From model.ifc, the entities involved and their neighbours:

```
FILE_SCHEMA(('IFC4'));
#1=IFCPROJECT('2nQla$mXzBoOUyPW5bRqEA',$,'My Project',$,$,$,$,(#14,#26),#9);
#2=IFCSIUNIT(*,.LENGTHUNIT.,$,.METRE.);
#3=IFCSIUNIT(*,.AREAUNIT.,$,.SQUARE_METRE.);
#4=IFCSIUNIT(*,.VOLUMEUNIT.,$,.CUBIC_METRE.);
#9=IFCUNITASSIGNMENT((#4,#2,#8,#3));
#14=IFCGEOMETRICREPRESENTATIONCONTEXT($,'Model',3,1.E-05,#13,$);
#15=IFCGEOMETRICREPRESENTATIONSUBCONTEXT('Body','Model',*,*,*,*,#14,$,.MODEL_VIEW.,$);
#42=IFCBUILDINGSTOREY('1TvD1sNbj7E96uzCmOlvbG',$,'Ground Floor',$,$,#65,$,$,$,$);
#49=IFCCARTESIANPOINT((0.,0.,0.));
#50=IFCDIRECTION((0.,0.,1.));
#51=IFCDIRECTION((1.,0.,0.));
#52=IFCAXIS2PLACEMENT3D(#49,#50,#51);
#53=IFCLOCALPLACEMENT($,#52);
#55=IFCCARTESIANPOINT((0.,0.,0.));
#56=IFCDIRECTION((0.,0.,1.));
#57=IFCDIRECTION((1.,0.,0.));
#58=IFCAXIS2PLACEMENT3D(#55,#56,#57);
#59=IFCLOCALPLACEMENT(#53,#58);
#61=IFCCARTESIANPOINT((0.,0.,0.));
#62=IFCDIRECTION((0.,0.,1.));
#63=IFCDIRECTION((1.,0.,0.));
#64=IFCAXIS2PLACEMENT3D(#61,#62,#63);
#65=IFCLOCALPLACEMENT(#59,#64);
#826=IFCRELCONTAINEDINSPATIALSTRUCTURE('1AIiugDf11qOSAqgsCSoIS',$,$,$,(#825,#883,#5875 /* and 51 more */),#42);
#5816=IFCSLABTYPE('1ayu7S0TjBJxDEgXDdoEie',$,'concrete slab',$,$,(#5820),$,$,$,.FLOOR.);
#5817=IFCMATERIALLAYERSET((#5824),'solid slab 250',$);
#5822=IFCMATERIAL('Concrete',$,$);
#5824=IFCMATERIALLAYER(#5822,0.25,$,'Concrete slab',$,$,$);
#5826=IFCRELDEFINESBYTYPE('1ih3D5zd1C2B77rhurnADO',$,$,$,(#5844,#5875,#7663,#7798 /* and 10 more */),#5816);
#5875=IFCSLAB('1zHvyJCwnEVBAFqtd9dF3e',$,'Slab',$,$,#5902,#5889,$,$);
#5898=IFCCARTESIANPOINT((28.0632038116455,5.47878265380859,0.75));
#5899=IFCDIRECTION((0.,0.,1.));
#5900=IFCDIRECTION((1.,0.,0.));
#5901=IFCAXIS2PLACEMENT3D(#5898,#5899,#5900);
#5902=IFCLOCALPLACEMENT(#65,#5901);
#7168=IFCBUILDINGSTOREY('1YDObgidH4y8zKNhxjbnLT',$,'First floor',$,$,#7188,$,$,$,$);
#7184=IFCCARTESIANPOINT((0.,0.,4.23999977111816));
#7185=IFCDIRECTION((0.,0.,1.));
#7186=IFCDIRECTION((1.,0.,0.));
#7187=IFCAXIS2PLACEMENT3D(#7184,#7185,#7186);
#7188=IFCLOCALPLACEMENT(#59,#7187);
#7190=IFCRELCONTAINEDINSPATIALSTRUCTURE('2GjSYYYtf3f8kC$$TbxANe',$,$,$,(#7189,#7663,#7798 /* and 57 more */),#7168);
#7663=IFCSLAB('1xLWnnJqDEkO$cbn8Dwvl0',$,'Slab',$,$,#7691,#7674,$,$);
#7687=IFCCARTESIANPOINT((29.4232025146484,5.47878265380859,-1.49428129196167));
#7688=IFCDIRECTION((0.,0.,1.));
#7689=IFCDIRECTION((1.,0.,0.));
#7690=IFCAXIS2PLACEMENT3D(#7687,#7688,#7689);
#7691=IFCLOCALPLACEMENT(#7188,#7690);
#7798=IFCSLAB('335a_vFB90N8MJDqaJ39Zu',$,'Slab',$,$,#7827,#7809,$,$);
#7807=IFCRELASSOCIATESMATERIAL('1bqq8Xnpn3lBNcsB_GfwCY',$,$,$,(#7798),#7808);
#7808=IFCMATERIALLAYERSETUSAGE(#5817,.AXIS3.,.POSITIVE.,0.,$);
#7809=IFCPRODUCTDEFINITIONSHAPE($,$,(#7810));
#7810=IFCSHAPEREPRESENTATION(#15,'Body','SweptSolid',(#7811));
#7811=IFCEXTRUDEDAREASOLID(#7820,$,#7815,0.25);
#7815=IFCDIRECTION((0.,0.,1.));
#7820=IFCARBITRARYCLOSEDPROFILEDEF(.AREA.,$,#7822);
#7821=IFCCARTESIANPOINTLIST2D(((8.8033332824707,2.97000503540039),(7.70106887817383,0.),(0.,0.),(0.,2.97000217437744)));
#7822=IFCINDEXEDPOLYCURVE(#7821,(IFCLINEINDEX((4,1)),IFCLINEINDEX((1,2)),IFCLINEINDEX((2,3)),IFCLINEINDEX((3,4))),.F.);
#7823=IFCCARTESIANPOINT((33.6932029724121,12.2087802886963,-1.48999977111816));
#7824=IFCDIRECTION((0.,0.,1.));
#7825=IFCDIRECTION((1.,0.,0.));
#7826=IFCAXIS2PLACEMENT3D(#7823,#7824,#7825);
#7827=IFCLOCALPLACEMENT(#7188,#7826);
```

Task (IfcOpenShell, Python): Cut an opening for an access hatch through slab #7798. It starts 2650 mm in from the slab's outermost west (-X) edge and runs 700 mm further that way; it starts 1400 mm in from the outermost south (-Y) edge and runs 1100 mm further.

```python
import numpy as np
import ifcopenshell
import ifcopenshell.api.feature
import ifcopenshell.api.geometry
import ifcopenshell.api.root
import ifcopenshell.geom
import ifcopenshell.util.placement
import ifcopenshell.util.representation
import ifcopenshell.util.shape
import ifcopenshell.util.unit

model = ifcopenshell.open("model.ifc")
unit_scale = ifcopenshell.util.unit.calculate_unit_scale(model)
settings = ifcopenshell.geom.settings()


def volume(element):
    """Net volume in cubic metres, openings subtracted."""
    shape = ifcopenshell.geom.create_shape(settings, element)
    return ifcopenshell.util.shape.get_volume(shape.geometry)


slab = model.by_guid("335a_vFB90N8MJDqaJ39Zu")
before = volume(slab)

# Extent in the slab's own axes, in metres. The edges named are its -X and -Y sides.
slab_shape = ifcopenshell.geom.create_shape(settings, slab)
vertices = ifcopenshell.util.shape.get_vertices(slab_shape.geometry)
x_min, y_min, bottom = vertices.min(axis=0)
top = vertices[:, 2].max()

opening = ifcopenshell.api.root.create_entity(model, ifc_class="IfcOpeningElement", name="Access hatch opening", predefined_type="OPENING")
context = ifcopenshell.util.representation.get_context(model, "Model", "Body", "MODEL_VIEW")
width, depth = 0.7, 1.1
outline = [(0.0, 0.0), (width, 0.0), (width, depth), (0.0, depth), (0.0, 0.0)]
# Overshoot both faces by 50 mm so the cut is clean.
shape = ifcopenshell.api.geometry.add_slab_representation(
    model, context=context, depth=top - bottom + 0.1, polyline=outline
)
ifcopenshell.api.geometry.assign_representation(model, product=opening, representation=shape)

matrix = ifcopenshell.util.placement.get_local_placement(slab.ObjectPlacement)
matrix[:, 3] = matrix @ np.append(np.array([x_min + 2.65, y_min + 1.4, bottom - 0.05]) / unit_scale, 1.0)
ifcopenshell.api.geometry.edit_object_placement(model, product=opening, matrix=matrix, is_si=False)
ifcopenshell.api.feature.add_feature(model, feature=opening, element=slab)

after = volume(slab)

print(f"slab volume {before:.3f} -> {after:.3f} m3")

model.write("model_v2.ifc")
```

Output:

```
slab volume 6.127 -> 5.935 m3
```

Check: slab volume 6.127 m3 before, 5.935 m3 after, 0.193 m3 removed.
